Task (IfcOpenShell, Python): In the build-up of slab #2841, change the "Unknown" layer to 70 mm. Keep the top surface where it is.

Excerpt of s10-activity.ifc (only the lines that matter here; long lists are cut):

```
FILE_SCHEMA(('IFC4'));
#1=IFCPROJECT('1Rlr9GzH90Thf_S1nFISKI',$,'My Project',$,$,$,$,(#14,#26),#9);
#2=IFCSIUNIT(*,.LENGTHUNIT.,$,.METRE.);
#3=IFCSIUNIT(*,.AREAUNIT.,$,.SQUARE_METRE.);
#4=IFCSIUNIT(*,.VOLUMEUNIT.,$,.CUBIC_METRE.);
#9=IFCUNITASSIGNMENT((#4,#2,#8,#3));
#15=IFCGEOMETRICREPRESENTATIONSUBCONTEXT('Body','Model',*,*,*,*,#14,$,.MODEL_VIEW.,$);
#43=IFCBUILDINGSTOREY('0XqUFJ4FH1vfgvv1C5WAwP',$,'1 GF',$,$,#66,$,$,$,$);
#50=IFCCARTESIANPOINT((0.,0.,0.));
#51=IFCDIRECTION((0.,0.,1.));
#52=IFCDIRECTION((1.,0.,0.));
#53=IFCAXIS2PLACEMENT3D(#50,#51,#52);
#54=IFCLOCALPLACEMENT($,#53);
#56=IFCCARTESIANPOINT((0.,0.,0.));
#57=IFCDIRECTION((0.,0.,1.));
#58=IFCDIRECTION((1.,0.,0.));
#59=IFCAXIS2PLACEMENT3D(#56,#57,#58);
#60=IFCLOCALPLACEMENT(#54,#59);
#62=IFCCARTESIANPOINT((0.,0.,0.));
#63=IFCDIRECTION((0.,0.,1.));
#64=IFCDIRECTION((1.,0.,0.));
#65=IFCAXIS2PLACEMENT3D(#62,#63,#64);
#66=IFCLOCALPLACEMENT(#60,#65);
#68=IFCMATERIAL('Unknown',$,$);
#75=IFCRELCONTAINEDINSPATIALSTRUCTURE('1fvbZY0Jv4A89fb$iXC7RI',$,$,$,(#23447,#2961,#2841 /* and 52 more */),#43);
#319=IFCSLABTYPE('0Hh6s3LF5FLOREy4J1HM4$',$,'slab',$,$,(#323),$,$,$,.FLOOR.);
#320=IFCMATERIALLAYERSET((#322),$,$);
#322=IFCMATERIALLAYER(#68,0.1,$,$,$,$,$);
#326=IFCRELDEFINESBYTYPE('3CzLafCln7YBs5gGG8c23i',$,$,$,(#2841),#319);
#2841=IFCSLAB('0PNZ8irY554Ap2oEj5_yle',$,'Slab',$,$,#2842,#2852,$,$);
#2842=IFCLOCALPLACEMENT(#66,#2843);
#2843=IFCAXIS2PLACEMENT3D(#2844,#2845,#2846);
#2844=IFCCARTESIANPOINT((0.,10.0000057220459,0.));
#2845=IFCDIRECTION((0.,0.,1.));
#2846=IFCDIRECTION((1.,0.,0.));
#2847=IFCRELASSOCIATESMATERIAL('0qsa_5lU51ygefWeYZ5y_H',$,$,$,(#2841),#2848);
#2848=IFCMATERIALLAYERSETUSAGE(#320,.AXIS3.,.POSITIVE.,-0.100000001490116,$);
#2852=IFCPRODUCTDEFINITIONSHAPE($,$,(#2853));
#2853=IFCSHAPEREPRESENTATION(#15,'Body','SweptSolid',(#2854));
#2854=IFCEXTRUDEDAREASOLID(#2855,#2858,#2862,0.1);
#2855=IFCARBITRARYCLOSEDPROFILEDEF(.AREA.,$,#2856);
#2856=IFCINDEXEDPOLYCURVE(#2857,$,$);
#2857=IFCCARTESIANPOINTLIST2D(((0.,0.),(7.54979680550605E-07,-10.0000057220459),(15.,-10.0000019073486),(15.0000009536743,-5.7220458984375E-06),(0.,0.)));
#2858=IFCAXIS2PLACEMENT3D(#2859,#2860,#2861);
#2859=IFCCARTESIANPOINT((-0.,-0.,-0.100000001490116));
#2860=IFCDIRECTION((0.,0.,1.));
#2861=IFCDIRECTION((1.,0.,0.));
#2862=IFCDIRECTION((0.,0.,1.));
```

```python
import ifcopenshell
import ifcopenshell.util.element
import ifcopenshell.util.representation
import ifcopenshell.util.unit

model = ifcopenshell.open("s10-activity.ifc")
unit_scale = ifcopenshell.util.unit.calculate_unit_scale(model)

layer_set = model.by_id(320)
layer = next(l for l in layer_set.MaterialLayers if l.Material and l.Material.Name == "Unknown")
change = 0.07 / unit_scale - layer.LayerThickness
layer.LayerThickness += change

# Geometry does not follow the layer set by itself.
slabs = [e for e in ifcopenshell.util.element.get_elements_by_material(model, layer_set) if e.is_a("IfcSlab")]
for slab in sorted(slabs, key=lambda e: e.id()):
    body = ifcopenshell.util.representation.get_representation(slab, "Model", "Body")
    solid = body.Items[0]
    old_depth = solid.Depth
    solid.Depth += change
    # Extruded upwards: lower the start of the extrusion so the top stays.
    x, y, z = solid.Position.Location.Coordinates
    solid.Position.Location = model.createIfcCartesianPoint((x, y, z - change))
    print(slab.id(), f"{old_depth:g} -> {solid.Depth:g}")

# The layers are counted up from the underside, which has moved.
for usage in {ifcopenshell.util.element.get_material(slab) for slab in slabs}:
    usage.OffsetFromReferenceLine -= change

model.write("s10-activity_rev.ifc")
```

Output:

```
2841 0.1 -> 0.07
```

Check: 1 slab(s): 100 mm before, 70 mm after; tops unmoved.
